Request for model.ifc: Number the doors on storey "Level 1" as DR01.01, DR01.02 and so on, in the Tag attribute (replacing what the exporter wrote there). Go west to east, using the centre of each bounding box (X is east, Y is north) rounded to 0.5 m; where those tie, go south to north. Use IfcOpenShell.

First a look at what the model holds.

```python
import ifcopenshell
import ifcopenshell.util.element
import ifcopenshell.util.placement

model = ifcopenshell.open("model.ifc")
print(model.schema)
storey = next(s for s in model.by_type("IfcBuildingStorey") if s.Name == "Level 1")
doors = [e for e in ifcopenshell.util.element.get_decomposition(storey) if e.is_a("IfcDoor")]
for e in sorted(doors, key=lambda e: e.id()):
    origin = ifcopenshell.util.placement.get_local_placement(e.ObjectPlacement)[:3, 3]
    print(e.id(), e.Tag, e.Name, origin.round(2) + 0.0, sep=" | ")
```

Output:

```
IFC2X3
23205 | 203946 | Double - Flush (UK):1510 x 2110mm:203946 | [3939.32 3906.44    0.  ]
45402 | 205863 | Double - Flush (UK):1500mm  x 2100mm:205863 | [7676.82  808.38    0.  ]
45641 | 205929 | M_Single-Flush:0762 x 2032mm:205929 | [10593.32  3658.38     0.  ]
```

```python
import ifcopenshell
import ifcopenshell.geom
import ifcopenshell.util.element
import ifcopenshell.util.shape

model = ifcopenshell.open("model.ifc")
settings = ifcopenshell.geom.settings()
settings.set("use-world-coords", True)


def centre(element):
    shape = ifcopenshell.geom.create_shape(settings, element)
    return ifcopenshell.util.shape.get_bbox_centroid(shape.geometry)


storey = next(s for s in model.by_type("IfcBuildingStorey") if s.Name == "Level 1")
doors = [e for e in ifcopenshell.util.element.get_decomposition(storey) if e.is_a("IfcDoor")]

# Insertion points can sit at a corner or the storey origin, so sort by the geometry (in metres).
centres = {e: centre(e) for e in doors}
doors.sort(key=lambda e: (round(centres[e][0] / 0.5), centres[e][1]))

for i, e in enumerate(doors, start=1):
    number = f"DR01.{i:02d}"
    e.Tag = number
    print(e.id(), number)

model.write("model_v2.ifc")
```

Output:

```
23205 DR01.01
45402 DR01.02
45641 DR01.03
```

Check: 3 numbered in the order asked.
